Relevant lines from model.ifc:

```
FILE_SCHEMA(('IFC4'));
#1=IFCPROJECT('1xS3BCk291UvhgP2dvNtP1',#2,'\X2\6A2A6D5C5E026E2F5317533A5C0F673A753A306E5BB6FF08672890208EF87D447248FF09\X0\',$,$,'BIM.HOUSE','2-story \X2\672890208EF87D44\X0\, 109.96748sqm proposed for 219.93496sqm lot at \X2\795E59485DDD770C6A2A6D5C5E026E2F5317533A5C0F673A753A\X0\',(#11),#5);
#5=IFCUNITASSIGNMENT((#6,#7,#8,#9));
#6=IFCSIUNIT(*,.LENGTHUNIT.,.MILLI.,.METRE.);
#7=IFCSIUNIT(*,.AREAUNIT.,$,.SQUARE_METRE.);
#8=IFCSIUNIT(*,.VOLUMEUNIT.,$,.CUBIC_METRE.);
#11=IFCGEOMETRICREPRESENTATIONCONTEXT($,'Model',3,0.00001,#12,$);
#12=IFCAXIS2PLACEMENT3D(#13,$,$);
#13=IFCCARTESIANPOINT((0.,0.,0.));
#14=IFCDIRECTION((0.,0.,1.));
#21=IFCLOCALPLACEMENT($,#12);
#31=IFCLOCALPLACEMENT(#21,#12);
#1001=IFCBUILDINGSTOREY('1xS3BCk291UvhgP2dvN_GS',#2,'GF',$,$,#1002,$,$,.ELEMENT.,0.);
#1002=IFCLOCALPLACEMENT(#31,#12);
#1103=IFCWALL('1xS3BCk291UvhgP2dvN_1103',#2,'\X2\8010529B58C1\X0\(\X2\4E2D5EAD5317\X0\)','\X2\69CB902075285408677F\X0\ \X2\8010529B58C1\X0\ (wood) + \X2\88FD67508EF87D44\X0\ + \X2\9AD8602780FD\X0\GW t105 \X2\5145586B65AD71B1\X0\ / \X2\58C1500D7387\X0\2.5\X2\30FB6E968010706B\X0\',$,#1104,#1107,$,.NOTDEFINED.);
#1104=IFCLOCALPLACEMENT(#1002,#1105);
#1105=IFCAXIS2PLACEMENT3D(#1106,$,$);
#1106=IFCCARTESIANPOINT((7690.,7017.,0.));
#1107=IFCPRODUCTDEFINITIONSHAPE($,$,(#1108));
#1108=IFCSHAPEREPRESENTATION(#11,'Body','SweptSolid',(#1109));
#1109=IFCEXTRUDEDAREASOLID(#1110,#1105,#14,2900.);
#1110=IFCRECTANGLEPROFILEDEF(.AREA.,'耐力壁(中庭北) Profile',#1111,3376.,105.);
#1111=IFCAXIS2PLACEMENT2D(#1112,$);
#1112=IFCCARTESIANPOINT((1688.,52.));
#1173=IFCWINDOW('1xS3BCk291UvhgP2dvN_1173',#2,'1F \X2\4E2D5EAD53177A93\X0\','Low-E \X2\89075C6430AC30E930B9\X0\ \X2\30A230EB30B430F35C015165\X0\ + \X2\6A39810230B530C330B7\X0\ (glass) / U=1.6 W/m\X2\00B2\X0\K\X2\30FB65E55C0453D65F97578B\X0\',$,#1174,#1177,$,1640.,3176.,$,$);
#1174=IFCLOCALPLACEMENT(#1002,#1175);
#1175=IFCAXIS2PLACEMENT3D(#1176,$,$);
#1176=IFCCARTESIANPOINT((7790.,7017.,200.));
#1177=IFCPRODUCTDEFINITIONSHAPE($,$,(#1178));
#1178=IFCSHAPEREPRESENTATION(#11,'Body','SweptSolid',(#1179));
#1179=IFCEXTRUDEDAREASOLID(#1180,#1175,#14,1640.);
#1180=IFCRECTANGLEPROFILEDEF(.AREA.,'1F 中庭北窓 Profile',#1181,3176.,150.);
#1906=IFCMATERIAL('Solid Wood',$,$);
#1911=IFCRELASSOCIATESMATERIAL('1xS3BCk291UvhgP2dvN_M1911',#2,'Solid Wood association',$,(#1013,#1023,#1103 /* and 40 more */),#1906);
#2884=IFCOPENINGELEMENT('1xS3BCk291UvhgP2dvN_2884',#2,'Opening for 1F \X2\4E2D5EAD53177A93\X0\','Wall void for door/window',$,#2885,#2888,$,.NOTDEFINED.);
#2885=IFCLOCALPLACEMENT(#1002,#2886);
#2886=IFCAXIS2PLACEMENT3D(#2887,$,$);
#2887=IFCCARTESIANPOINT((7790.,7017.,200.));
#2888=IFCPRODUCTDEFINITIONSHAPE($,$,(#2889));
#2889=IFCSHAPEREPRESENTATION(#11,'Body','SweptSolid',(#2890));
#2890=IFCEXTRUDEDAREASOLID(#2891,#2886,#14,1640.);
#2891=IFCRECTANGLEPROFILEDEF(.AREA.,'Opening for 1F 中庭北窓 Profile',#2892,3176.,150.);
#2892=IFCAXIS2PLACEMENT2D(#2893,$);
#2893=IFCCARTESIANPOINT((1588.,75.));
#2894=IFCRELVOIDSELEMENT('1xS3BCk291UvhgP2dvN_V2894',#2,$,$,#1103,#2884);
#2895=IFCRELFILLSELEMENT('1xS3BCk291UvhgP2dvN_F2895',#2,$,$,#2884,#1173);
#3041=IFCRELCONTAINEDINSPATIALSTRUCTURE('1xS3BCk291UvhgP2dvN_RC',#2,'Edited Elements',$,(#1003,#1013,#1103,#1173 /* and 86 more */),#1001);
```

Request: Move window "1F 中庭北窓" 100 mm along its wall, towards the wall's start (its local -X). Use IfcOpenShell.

```python
import ifcopenshell
import ifcopenshell.api.geometry
import ifcopenshell.util.placement
import ifcopenshell.util.unit

model = ifcopenshell.open("model.ifc")
unit_scale = ifcopenshell.util.unit.calculate_unit_scale(model)

window = model.by_id(1173)
opening = window.FillsVoids[0].RelatingOpeningElement
wall = opening.VoidsElements[0].RelatingBuildingElement

wall_matrix = ifcopenshell.util.placement.get_local_placement(wall.ObjectPlacement)
shift = wall_matrix[:3, 0] * -0.1 / unit_scale
before = ifcopenshell.util.placement.get_local_placement(window.ObjectPlacement)[:3, 3].copy()

# The window is not placed relative to its opening, so move both.
for product in (opening, window):
    matrix = ifcopenshell.util.placement.get_local_placement(product.ObjectPlacement)
    matrix[:3, 3] += shift
    ifcopenshell.api.geometry.edit_object_placement(model, product=product, matrix=matrix, is_si=False)

after = ifcopenshell.util.placement.get_local_placement(window.ObjectPlacement)[:3, 3]
print("window moved by", (after - before).round(3) + 0.0)

model.write("model_updated.ifc")
```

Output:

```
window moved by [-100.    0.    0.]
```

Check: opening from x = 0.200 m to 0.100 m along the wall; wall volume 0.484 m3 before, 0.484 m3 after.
